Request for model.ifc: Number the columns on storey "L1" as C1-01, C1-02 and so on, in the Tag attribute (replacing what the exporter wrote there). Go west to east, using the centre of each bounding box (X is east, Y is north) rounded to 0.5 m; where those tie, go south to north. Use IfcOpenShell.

First a look at what the model holds.

```python
import ifcopenshell
import ifcopenshell.util.element
import ifcopenshell.util.placement

model = ifcopenshell.open("model.ifc")
print(model.schema)
storey = next(s for s in model.by_type("IfcBuildingStorey") if s.Name == "L1")
columns = [e for e in ifcopenshell.util.element.get_decomposition(storey) if e.is_a("IfcColumn")]
for e in sorted(columns, key=lambda e: e.id()):
    origin = ifcopenshell.util.placement.get_local_placement(e.ObjectPlacement)[:3, 3]
    print(e.id(), e.Tag, e.Name, origin.round(2) + 0.0, sep=" | ")
```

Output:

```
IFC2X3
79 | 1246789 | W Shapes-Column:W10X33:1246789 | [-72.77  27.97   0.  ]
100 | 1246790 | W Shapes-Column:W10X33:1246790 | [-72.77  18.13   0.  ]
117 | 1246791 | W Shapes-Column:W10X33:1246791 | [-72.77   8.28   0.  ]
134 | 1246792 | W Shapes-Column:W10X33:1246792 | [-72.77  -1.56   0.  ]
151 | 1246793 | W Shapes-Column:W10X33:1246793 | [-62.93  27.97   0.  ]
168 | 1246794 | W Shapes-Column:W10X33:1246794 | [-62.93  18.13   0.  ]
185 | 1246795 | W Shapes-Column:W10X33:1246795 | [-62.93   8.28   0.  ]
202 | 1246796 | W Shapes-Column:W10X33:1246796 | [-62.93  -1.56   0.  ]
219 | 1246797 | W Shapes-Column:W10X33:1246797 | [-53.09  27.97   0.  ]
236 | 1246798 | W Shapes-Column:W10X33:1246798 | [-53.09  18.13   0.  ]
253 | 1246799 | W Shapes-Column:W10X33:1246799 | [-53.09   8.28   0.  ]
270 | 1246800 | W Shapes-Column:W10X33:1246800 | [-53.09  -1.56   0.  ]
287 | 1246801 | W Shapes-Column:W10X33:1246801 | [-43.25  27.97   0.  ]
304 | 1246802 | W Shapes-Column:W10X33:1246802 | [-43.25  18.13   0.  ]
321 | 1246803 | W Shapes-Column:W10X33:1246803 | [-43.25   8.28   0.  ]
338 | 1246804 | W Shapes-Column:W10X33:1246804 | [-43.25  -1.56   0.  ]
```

```python
import ifcopenshell
import ifcopenshell.geom
import ifcopenshell.util.element
import ifcopenshell.util.shape

model = ifcopenshell.open("model.ifc")
settings = ifcopenshell.geom.settings()
settings.set("use-world-coords", True)


def centre(element):
    shape = ifcopenshell.geom.create_shape(settings, element)
    return ifcopenshell.util.shape.get_bbox_centroid(shape.geometry)


storey = next(s for s in model.by_type("IfcBuildingStorey") if s.Name == "L1")
columns = [e for e in ifcopenshell.util.element.get_decomposition(storey) if e.is_a("IfcColumn")]

# Insertion points can sit at a corner or the storey origin, so sort by the geometry (in metres).
centres = {e: centre(e) for e in columns}
columns.sort(key=lambda e: (round(centres[e][0] / 0.5), centres[e][1]))

for i, e in enumerate(columns, start=1):
    number = f"C1-{i:02d}"
    e.Tag = number
    print(e.id(), number)

model.write("model_v2.ifc")
```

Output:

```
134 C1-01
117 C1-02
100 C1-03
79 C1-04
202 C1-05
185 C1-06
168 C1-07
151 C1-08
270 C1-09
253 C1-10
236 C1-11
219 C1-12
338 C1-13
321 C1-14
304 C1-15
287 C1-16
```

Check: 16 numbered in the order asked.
